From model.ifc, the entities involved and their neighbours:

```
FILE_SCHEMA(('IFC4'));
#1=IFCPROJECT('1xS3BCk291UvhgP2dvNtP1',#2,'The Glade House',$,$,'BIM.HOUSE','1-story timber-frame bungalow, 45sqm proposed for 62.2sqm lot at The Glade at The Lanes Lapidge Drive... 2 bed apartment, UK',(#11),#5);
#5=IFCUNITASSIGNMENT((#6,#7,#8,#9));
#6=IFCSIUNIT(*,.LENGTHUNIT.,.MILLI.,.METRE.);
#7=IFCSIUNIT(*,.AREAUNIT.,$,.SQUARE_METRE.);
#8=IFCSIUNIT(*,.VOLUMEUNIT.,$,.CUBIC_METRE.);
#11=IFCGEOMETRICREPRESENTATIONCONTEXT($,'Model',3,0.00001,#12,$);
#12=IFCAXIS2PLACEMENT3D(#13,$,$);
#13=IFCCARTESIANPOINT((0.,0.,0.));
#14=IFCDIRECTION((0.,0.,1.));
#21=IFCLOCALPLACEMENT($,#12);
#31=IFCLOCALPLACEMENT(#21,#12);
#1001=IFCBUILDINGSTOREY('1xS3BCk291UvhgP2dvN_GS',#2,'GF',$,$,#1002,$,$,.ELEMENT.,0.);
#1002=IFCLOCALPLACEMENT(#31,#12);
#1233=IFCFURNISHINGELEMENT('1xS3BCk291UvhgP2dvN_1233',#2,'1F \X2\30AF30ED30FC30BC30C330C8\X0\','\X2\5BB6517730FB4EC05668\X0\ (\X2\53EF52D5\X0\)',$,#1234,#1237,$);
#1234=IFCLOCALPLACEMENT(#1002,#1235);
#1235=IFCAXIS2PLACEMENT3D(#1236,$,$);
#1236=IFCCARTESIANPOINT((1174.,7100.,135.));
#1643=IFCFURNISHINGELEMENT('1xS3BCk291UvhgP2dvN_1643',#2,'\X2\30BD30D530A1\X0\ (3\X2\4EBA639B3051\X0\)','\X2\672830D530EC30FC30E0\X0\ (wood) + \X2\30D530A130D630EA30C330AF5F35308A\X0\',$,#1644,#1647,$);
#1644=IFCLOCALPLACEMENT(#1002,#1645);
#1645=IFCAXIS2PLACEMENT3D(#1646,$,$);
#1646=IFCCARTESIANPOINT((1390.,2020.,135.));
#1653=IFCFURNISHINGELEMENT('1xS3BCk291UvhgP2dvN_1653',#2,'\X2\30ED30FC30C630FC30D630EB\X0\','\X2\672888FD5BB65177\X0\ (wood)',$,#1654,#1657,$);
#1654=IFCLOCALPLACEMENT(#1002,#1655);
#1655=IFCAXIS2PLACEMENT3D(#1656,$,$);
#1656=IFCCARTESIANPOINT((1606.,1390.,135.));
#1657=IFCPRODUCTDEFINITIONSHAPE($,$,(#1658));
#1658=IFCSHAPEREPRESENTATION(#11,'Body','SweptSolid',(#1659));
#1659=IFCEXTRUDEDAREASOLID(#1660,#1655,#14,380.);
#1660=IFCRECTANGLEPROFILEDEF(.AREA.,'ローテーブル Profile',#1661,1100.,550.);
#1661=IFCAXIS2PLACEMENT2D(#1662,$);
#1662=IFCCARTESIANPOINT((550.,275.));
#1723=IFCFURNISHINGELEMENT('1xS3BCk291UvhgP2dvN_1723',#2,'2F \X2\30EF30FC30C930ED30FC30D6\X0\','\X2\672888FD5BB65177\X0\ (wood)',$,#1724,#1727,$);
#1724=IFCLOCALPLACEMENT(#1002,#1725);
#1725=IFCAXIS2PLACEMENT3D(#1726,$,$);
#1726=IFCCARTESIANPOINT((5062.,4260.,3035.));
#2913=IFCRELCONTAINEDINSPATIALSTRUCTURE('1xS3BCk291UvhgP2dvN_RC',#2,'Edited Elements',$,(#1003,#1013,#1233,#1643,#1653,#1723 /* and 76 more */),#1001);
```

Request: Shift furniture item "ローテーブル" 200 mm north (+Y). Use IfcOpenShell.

```python
import ifcopenshell
import ifcopenshell.api.geometry
import ifcopenshell.util.placement
import ifcopenshell.util.unit

model = ifcopenshell.open("model.ifc")
unit_scale = ifcopenshell.util.unit.calculate_unit_scale(model)

item = model.by_id(1653)
matrix = ifcopenshell.util.placement.get_local_placement(item.ObjectPlacement)
matrix[1, 3] += 0.2 / unit_scale
ifcopenshell.api.geometry.edit_object_placement(model, product=item, matrix=matrix, is_si=False)

print(ifcopenshell.util.placement.get_local_placement(item.ObjectPlacement).round(3) + 0.0)

model.write("model_rev.ifc")
```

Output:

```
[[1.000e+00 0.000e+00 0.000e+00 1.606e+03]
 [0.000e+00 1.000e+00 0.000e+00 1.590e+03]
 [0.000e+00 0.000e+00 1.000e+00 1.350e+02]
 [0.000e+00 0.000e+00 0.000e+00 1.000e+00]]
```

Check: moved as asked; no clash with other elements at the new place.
